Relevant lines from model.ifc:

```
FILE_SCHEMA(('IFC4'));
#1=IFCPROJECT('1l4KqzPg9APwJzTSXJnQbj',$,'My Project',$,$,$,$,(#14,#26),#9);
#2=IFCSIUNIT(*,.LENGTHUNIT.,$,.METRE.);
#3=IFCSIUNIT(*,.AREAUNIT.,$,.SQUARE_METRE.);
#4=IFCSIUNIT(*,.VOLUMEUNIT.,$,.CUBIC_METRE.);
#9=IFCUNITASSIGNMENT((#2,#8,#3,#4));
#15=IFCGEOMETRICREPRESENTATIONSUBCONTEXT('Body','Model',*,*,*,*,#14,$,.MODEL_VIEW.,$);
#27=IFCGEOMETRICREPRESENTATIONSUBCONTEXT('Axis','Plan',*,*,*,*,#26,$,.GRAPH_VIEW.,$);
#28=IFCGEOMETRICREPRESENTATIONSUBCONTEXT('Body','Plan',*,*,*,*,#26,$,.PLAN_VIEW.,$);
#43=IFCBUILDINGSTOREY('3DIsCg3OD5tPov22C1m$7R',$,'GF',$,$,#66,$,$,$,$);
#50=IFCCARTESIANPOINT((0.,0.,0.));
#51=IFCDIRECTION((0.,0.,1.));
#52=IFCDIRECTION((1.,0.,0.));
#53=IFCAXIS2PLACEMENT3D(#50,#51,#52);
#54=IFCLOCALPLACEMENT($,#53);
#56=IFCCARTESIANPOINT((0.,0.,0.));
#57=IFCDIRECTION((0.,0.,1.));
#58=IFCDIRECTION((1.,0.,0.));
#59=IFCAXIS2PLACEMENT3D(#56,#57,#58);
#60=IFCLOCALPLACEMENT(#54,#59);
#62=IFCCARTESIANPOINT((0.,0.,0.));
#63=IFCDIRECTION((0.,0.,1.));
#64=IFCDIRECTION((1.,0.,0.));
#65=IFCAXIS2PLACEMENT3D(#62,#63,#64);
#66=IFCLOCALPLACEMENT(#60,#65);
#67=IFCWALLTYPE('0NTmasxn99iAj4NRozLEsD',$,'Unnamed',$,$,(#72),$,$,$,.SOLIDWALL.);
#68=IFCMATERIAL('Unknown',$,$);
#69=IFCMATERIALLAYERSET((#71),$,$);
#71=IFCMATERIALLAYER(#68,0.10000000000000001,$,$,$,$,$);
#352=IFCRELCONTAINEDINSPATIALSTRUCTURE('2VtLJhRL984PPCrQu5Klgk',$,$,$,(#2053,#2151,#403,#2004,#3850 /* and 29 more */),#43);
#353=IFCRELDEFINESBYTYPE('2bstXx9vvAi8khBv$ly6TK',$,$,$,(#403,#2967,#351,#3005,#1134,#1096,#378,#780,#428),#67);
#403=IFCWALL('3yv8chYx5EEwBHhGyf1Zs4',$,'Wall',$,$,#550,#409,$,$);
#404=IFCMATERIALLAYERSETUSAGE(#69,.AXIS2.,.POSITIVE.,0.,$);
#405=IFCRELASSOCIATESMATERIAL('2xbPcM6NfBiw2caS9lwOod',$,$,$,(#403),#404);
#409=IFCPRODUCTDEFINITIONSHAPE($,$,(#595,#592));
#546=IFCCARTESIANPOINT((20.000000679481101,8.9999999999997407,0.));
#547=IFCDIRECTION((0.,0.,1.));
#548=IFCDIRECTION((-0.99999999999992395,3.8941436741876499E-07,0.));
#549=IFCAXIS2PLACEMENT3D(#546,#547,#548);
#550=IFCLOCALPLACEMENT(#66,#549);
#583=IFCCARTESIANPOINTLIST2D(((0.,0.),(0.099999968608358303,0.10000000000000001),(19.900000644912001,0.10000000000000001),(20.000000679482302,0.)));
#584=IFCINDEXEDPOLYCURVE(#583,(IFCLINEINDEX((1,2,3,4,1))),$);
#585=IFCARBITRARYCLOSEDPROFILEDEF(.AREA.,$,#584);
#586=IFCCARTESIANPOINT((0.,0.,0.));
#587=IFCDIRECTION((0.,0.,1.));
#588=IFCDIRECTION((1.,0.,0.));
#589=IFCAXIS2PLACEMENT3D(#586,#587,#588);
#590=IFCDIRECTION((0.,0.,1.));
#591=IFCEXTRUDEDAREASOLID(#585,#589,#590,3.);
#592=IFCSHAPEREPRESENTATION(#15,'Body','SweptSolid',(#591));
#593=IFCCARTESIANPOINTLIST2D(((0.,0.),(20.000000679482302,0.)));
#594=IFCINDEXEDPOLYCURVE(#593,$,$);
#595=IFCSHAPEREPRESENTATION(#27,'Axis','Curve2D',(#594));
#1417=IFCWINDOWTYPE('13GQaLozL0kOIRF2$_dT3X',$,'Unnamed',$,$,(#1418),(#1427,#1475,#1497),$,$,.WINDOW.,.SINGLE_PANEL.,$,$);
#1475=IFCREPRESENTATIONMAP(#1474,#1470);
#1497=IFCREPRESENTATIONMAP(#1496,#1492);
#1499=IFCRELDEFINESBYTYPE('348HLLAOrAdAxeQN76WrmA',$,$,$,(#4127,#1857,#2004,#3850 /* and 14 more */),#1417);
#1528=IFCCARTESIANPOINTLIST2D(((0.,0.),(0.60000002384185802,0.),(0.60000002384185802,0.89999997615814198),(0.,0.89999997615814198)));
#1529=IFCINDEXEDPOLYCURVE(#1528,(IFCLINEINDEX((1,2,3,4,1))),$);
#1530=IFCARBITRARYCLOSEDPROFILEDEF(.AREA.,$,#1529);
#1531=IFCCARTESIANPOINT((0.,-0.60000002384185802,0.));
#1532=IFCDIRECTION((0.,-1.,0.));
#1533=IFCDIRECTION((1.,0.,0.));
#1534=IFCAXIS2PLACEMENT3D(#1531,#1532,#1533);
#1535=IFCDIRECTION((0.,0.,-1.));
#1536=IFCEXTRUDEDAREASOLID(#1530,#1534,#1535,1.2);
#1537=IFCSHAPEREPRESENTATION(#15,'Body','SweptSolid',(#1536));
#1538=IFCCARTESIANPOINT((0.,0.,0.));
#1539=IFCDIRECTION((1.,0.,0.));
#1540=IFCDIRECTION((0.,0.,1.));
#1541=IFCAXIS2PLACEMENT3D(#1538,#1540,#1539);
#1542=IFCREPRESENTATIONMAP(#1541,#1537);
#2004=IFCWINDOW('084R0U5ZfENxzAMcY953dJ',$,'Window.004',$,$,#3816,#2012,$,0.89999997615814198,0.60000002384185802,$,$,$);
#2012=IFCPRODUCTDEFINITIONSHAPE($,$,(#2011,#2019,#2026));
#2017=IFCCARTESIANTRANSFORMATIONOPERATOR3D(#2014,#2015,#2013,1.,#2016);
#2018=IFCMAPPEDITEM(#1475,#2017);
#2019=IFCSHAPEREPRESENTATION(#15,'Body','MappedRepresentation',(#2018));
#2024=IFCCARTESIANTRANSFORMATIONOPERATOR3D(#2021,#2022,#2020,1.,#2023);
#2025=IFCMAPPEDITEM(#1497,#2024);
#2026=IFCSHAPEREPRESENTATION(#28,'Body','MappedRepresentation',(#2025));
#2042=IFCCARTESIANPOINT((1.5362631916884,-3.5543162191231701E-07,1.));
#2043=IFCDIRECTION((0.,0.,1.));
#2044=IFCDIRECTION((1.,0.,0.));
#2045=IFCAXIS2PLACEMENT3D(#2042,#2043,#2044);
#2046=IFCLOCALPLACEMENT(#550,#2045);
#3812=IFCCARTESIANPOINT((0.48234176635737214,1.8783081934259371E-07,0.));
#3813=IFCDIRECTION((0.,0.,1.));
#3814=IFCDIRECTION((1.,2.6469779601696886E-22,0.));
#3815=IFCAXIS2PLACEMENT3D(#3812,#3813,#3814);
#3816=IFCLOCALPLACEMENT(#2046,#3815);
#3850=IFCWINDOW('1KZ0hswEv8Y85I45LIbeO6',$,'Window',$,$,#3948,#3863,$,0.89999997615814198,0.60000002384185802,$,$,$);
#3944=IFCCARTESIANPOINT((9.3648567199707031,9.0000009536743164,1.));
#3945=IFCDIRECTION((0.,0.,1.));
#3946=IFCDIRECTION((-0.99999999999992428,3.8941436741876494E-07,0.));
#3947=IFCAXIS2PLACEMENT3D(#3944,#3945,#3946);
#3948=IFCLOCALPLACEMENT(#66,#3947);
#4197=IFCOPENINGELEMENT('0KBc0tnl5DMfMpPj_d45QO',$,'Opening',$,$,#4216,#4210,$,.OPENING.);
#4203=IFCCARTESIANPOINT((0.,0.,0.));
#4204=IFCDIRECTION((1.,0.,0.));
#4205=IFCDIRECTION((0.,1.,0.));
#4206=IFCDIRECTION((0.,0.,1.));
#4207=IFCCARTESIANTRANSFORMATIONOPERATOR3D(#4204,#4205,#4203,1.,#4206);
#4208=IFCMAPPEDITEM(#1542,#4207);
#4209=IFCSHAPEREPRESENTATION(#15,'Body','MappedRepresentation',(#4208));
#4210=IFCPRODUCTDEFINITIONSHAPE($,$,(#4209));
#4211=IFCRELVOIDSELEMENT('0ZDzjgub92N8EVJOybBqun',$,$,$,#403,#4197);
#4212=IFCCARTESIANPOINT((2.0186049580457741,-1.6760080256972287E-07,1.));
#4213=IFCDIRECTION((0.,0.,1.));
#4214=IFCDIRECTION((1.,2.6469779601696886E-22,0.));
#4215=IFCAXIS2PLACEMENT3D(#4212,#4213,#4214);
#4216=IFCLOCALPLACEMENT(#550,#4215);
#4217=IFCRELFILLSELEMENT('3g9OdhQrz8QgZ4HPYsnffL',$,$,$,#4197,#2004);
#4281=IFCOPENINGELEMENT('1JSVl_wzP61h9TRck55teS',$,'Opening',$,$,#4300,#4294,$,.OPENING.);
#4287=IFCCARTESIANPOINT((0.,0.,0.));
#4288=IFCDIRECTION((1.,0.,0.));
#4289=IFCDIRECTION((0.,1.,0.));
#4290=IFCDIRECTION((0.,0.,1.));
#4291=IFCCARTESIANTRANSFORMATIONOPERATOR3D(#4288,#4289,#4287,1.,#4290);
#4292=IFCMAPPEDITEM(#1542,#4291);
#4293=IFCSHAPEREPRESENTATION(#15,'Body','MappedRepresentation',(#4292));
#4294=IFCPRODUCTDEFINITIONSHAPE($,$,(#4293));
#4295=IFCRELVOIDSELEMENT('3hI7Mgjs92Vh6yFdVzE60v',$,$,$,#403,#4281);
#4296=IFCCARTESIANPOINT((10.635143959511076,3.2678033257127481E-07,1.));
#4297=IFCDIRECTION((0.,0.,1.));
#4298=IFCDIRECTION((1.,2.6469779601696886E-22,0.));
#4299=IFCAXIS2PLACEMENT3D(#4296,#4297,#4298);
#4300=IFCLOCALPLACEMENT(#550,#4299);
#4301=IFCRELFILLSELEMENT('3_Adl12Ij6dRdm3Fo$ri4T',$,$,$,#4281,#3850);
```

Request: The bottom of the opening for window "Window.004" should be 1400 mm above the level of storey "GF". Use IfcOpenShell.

```python
import numpy as np
import ifcopenshell
import ifcopenshell.api.geometry
import ifcopenshell.geom
import ifcopenshell.util.element
import ifcopenshell.util.placement
import ifcopenshell.util.shape
import ifcopenshell.util.unit

model = ifcopenshell.open("model.ifc")
unit_scale = ifcopenshell.util.unit.calculate_unit_scale(model)

window = model.by_id(2004)
opening = window.FillsVoids[0].RelatingOpeningElement
storey = ifcopenshell.util.element.get_container(window, ifc_class="IfcBuildingStorey")
level = ifcopenshell.util.placement.get_local_placement(storey.ObjectPlacement)[2, 3]

# The opening's origin need not be at the sill, so measure its lowest point.
shape = ifcopenshell.geom.create_shape(ifcopenshell.geom.settings(), opening)
bottom = ifcopenshell.util.shape.get_shape_bottom_elevation(shape, shape.geometry) / unit_scale
dz = level + 1.4 - bottom

shift = np.array([0.0, 0.0, dz])
# The window is not placed relative to its opening, so move both.
for product in (opening, window):
    matrix = ifcopenshell.util.placement.get_local_placement(product.ObjectPlacement)
    matrix[:3, 3] += shift
    ifcopenshell.api.geometry.edit_object_placement(model, product=product, matrix=matrix, is_si=False)

print(f"moved by {dz * unit_scale:+.3f} m")

model.write("model_v2.ifc")
```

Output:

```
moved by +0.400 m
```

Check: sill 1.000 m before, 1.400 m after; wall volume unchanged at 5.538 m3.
